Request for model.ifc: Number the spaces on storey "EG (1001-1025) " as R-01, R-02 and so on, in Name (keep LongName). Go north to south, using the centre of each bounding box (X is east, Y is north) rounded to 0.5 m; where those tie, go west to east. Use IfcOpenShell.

First a look at what the model holds.

```python
import ifcopenshell
import ifcopenshell.util.element
import ifcopenshell.util.placement

model = ifcopenshell.open("model.ifc")
print(model.schema)
storey = next(s for s in model.by_type("IfcBuildingStorey") if s.Name == "EG (1001-1025) ")
spaces = [e for e in ifcopenshell.util.element.get_decomposition(storey) if e.is_a("IfcSpace")]
for e in sorted(spaces, key=lambda e: e.id()):
    origin = ifcopenshell.util.placement.get_local_placement(e.ObjectPlacement)[:3, 3]
    print(e.id(), e.Name, e.LongName, origin.round(2) + 0.0, sep=" | ")
```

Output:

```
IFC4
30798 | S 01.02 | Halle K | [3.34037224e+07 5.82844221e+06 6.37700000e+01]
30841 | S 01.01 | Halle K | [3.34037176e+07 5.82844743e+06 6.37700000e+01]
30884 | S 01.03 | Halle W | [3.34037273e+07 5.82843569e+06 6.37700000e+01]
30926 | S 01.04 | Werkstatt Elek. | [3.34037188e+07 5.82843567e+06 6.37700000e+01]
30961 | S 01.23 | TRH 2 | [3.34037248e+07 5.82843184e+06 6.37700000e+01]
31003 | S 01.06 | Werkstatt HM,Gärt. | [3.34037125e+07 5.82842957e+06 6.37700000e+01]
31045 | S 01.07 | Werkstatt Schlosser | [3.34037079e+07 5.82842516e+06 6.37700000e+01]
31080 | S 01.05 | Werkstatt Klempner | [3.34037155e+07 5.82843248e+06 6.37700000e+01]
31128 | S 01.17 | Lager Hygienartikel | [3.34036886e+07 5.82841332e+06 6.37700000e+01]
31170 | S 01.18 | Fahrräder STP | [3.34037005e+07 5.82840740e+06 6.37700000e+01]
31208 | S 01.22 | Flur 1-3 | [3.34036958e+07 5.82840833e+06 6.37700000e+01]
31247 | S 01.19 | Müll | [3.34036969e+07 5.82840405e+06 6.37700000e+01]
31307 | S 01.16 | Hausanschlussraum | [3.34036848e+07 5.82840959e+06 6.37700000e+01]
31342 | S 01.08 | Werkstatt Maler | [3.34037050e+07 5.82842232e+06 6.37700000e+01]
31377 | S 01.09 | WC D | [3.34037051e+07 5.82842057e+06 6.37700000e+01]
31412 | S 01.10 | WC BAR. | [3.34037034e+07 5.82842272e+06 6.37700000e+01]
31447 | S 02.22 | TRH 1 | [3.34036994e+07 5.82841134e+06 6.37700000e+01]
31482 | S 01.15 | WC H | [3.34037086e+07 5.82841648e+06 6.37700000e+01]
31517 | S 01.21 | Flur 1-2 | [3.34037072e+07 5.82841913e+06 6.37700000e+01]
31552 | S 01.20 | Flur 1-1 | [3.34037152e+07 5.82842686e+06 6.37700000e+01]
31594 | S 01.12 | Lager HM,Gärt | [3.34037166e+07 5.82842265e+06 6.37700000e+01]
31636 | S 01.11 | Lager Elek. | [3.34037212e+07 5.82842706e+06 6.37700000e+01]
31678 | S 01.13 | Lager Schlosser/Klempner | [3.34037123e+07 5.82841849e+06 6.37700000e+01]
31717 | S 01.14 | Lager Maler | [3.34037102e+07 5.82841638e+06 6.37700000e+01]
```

```python
import ifcopenshell
import ifcopenshell.geom
import ifcopenshell.util.element
import ifcopenshell.util.shape

model = ifcopenshell.open("model.ifc")
settings = ifcopenshell.geom.settings()
settings.set("use-world-coords", True)


def centre(element):
    shape = ifcopenshell.geom.create_shape(settings, element)
    return ifcopenshell.util.shape.get_bbox_centroid(shape.geometry)


storey = next(s for s in model.by_type("IfcBuildingStorey") if s.Name == "EG (1001-1025) ")
spaces = [e for e in ifcopenshell.util.element.get_decomposition(storey) if e.is_a("IfcSpace")]

# Insertion points can sit at a corner or the storey origin, so sort by the geometry (in metres).
centres = {e: centre(e) for e in spaces}
spaces.sort(key=lambda e: (-round(centres[e][1] / 0.5), centres[e][0]))

for i, e in enumerate(spaces, start=1):
    number = f"R-{i:02d}"
    e.Name = number
    print(e.id(), number)

model.write("model_edited.ifc")
```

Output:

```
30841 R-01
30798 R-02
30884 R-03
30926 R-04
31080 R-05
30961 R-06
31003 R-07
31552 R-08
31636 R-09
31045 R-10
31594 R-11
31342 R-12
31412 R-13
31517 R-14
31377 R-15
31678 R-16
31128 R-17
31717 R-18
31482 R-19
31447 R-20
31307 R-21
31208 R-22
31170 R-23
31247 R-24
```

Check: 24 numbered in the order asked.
